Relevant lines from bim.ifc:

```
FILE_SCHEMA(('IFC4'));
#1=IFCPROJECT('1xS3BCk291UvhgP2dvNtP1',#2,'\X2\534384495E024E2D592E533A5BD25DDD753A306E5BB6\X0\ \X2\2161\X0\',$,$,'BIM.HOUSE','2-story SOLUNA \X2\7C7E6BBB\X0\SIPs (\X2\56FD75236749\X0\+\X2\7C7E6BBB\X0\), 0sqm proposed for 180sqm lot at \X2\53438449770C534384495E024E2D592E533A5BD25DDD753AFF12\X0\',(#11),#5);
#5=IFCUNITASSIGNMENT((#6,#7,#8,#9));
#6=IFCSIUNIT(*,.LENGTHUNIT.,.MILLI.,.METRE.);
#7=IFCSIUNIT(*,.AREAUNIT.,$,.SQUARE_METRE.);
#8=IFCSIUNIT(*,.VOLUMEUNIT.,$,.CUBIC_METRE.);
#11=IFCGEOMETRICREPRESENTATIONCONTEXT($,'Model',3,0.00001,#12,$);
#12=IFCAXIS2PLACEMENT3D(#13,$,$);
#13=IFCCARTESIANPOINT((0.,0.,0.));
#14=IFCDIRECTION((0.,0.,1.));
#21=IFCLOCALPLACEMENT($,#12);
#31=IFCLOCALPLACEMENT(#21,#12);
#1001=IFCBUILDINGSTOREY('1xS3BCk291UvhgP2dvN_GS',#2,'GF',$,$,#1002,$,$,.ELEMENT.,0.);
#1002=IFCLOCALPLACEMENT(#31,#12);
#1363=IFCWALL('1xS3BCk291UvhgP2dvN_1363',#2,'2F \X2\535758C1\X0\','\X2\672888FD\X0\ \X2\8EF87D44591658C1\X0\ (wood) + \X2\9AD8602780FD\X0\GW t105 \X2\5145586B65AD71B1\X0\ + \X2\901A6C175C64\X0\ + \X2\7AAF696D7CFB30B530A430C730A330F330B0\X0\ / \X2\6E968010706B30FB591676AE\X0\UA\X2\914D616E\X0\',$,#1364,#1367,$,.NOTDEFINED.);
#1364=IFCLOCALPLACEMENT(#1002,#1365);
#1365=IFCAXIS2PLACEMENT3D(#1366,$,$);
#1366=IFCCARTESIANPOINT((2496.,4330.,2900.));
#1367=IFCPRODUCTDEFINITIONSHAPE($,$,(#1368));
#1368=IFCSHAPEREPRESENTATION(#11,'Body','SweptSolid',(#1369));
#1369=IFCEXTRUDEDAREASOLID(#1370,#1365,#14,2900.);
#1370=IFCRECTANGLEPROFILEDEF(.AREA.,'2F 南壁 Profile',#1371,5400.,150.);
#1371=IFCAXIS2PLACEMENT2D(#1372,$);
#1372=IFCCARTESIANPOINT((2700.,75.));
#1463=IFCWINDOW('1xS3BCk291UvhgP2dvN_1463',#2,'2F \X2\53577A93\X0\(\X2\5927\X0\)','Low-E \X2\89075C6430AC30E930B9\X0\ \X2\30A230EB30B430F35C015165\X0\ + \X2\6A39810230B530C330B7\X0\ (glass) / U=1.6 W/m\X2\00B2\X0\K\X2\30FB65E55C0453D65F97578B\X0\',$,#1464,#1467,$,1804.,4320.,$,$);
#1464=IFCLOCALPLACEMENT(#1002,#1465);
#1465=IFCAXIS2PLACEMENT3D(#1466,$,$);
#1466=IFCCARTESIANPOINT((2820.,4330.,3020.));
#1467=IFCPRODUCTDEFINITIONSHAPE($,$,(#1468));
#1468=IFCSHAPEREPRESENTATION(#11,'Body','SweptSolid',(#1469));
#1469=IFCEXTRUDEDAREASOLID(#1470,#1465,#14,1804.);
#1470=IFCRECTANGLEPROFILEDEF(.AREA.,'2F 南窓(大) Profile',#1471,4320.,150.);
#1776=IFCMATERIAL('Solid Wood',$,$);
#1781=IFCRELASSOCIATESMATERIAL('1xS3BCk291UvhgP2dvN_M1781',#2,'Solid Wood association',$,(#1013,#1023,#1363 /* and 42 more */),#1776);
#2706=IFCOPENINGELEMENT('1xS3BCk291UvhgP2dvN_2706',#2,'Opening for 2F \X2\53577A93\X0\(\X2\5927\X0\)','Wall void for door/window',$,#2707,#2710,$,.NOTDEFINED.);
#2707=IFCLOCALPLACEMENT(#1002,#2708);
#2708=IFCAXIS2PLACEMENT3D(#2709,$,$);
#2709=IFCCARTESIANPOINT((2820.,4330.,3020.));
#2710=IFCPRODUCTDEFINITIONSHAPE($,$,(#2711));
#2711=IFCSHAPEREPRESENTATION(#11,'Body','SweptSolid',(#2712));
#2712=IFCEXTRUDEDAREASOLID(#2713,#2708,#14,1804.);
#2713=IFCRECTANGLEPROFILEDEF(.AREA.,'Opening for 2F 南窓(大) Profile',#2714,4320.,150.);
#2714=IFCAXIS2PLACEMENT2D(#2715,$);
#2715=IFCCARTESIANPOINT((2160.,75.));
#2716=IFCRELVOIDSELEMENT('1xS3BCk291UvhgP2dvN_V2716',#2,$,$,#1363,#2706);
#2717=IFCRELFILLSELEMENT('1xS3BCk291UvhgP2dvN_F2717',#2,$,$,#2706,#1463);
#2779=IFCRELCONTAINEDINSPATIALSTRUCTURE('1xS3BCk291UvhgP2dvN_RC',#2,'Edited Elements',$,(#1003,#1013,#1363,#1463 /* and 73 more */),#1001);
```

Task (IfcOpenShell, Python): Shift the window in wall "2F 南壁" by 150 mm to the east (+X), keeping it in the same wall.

```python
import ifcopenshell
import ifcopenshell.api.geometry
import ifcopenshell.util.placement

model = ifcopenshell.open("bim.ifc")

window = model.by_id(1463)
opening = window.FillsVoids[0].RelatingOpeningElement
wall = opening.VoidsElements[0].RelatingBuildingElement

wall_matrix = ifcopenshell.util.placement.get_local_placement(wall.ObjectPlacement)
shift = wall_matrix[:3, 0] * 150.0
before = ifcopenshell.util.placement.get_local_placement(window.ObjectPlacement)[:3, 3].copy()

# The window is not placed relative to its opening, so move both.
for product in (opening, window):
    matrix = ifcopenshell.util.placement.get_local_placement(product.ObjectPlacement)
    matrix[:3, 3] += shift
    ifcopenshell.api.geometry.edit_object_placement(model, product=product, matrix=matrix, is_si=False)

after = ifcopenshell.util.placement.get_local_placement(window.ObjectPlacement)[:3, 3]
print("window moved by", (after - before).round(3) + 0.0)

model.write("bim_edited.ifc")
```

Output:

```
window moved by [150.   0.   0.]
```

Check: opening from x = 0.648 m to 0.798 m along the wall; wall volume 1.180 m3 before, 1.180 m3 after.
